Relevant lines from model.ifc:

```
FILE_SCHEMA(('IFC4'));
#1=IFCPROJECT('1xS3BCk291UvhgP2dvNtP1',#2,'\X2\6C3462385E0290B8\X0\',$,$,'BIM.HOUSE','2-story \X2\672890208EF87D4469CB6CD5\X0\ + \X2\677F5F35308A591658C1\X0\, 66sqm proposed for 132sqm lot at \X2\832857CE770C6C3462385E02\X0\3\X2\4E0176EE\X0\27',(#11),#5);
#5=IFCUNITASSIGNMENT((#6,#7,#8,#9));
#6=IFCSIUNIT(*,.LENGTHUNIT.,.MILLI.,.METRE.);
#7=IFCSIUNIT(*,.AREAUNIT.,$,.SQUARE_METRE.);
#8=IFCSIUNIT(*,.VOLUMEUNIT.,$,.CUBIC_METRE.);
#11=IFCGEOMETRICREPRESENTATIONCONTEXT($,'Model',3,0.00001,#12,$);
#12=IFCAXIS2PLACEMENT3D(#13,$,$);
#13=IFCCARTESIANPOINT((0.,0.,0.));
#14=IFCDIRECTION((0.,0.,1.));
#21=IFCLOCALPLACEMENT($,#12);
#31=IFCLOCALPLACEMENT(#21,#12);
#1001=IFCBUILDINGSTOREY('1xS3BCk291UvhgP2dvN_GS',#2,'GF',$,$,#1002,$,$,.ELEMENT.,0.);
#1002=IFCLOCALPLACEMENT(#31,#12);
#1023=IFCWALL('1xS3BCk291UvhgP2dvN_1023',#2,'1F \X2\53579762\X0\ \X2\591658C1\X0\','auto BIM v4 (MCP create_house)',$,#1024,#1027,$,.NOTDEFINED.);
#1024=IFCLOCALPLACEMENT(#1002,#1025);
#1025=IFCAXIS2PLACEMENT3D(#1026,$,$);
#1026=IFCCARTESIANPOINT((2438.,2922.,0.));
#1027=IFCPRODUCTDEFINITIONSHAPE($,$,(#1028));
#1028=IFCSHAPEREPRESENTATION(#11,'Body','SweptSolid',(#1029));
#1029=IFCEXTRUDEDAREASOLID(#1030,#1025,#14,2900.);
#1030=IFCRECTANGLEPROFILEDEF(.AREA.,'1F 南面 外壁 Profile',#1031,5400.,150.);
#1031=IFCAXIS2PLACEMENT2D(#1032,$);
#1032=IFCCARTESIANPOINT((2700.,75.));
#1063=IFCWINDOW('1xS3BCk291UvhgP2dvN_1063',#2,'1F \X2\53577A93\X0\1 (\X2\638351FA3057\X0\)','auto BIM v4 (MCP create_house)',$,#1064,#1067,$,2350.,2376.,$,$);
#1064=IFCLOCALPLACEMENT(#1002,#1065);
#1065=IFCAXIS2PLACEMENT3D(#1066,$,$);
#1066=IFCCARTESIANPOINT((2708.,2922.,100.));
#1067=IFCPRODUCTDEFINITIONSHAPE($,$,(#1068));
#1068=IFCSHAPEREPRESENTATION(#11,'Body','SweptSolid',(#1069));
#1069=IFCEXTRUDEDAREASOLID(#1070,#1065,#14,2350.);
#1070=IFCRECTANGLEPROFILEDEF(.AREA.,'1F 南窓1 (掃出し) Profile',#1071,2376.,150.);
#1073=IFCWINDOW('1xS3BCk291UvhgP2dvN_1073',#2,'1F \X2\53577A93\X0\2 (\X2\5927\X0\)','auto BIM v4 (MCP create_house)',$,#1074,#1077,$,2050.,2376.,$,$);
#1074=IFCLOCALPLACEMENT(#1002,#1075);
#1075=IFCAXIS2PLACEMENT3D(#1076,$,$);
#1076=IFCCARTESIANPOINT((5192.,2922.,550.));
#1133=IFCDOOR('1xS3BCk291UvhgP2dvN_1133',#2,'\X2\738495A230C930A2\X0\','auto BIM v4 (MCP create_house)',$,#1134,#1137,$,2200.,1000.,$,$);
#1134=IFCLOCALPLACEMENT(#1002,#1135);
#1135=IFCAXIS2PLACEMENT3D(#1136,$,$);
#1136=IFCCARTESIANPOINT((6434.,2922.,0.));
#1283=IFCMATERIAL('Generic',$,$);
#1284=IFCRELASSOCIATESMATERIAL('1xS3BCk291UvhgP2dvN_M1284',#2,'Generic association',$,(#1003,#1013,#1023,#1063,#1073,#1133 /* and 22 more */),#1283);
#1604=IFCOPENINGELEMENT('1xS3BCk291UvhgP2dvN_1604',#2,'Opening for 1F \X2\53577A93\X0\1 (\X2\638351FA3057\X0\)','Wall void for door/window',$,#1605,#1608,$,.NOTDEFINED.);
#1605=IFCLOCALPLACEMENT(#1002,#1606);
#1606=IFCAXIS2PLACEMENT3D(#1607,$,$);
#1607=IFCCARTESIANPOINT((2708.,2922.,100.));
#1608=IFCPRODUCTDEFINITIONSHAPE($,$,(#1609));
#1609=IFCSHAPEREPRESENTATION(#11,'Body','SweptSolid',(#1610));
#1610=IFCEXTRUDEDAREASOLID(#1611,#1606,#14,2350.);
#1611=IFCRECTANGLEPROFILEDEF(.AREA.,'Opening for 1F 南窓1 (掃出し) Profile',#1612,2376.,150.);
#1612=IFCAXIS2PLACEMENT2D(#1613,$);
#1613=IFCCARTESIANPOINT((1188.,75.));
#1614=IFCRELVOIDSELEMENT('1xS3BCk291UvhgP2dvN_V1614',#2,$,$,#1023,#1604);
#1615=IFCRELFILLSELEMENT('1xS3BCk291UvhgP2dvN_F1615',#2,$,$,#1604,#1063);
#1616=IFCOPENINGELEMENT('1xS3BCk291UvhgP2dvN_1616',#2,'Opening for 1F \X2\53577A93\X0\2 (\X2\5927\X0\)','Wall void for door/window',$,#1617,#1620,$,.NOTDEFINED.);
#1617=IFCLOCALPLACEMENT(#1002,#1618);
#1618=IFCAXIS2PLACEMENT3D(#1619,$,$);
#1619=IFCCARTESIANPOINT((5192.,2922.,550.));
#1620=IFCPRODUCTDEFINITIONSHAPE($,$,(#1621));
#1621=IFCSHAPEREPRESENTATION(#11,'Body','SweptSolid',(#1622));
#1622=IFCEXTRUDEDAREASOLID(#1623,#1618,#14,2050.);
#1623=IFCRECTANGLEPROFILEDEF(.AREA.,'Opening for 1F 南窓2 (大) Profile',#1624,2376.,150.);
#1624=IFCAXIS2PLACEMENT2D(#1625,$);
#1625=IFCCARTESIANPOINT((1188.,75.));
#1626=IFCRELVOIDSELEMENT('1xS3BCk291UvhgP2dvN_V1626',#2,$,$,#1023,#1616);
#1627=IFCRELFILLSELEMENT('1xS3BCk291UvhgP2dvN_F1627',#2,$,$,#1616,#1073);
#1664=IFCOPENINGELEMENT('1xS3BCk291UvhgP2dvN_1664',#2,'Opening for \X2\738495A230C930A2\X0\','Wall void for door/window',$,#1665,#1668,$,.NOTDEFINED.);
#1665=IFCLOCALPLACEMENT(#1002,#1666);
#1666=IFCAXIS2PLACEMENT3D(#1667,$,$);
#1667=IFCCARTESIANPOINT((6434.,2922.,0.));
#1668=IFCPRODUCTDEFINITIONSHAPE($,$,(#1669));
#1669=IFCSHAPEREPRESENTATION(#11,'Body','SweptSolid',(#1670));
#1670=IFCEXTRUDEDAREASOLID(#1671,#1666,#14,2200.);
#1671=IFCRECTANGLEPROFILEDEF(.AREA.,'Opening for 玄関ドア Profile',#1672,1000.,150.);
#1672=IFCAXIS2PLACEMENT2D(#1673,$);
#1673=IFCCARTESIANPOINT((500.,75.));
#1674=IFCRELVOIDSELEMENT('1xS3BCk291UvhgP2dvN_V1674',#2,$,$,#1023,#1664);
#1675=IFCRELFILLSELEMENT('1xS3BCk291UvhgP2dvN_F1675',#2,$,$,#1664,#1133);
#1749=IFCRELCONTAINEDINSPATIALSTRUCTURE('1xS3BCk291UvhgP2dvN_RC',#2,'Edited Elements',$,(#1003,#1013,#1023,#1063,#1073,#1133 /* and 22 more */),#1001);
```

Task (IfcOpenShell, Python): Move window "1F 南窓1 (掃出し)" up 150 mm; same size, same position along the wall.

```python
import numpy as np
import ifcopenshell
import ifcopenshell.api.geometry
import ifcopenshell.util.placement
import ifcopenshell.util.unit

model = ifcopenshell.open("model.ifc")
unit_scale = ifcopenshell.util.unit.calculate_unit_scale(model)

window = model.by_guid("1xS3BCk291UvhgP2dvN_1063")
opening = window.FillsVoids[0].RelatingOpeningElement
dz = 150.0

shift = np.array([0.0, 0.0, dz])
# The window is not placed relative to its opening, so move both.
for product in (opening, window):
    matrix = ifcopenshell.util.placement.get_local_placement(product.ObjectPlacement)
    matrix[:3, 3] += shift
    ifcopenshell.api.geometry.edit_object_placement(model, product=product, matrix=matrix, is_si=False)

print(f"moved by {dz * unit_scale:+.3f} m")

model.write("model_updated.ifc")
```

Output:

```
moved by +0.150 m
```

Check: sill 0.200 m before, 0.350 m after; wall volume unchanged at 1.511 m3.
